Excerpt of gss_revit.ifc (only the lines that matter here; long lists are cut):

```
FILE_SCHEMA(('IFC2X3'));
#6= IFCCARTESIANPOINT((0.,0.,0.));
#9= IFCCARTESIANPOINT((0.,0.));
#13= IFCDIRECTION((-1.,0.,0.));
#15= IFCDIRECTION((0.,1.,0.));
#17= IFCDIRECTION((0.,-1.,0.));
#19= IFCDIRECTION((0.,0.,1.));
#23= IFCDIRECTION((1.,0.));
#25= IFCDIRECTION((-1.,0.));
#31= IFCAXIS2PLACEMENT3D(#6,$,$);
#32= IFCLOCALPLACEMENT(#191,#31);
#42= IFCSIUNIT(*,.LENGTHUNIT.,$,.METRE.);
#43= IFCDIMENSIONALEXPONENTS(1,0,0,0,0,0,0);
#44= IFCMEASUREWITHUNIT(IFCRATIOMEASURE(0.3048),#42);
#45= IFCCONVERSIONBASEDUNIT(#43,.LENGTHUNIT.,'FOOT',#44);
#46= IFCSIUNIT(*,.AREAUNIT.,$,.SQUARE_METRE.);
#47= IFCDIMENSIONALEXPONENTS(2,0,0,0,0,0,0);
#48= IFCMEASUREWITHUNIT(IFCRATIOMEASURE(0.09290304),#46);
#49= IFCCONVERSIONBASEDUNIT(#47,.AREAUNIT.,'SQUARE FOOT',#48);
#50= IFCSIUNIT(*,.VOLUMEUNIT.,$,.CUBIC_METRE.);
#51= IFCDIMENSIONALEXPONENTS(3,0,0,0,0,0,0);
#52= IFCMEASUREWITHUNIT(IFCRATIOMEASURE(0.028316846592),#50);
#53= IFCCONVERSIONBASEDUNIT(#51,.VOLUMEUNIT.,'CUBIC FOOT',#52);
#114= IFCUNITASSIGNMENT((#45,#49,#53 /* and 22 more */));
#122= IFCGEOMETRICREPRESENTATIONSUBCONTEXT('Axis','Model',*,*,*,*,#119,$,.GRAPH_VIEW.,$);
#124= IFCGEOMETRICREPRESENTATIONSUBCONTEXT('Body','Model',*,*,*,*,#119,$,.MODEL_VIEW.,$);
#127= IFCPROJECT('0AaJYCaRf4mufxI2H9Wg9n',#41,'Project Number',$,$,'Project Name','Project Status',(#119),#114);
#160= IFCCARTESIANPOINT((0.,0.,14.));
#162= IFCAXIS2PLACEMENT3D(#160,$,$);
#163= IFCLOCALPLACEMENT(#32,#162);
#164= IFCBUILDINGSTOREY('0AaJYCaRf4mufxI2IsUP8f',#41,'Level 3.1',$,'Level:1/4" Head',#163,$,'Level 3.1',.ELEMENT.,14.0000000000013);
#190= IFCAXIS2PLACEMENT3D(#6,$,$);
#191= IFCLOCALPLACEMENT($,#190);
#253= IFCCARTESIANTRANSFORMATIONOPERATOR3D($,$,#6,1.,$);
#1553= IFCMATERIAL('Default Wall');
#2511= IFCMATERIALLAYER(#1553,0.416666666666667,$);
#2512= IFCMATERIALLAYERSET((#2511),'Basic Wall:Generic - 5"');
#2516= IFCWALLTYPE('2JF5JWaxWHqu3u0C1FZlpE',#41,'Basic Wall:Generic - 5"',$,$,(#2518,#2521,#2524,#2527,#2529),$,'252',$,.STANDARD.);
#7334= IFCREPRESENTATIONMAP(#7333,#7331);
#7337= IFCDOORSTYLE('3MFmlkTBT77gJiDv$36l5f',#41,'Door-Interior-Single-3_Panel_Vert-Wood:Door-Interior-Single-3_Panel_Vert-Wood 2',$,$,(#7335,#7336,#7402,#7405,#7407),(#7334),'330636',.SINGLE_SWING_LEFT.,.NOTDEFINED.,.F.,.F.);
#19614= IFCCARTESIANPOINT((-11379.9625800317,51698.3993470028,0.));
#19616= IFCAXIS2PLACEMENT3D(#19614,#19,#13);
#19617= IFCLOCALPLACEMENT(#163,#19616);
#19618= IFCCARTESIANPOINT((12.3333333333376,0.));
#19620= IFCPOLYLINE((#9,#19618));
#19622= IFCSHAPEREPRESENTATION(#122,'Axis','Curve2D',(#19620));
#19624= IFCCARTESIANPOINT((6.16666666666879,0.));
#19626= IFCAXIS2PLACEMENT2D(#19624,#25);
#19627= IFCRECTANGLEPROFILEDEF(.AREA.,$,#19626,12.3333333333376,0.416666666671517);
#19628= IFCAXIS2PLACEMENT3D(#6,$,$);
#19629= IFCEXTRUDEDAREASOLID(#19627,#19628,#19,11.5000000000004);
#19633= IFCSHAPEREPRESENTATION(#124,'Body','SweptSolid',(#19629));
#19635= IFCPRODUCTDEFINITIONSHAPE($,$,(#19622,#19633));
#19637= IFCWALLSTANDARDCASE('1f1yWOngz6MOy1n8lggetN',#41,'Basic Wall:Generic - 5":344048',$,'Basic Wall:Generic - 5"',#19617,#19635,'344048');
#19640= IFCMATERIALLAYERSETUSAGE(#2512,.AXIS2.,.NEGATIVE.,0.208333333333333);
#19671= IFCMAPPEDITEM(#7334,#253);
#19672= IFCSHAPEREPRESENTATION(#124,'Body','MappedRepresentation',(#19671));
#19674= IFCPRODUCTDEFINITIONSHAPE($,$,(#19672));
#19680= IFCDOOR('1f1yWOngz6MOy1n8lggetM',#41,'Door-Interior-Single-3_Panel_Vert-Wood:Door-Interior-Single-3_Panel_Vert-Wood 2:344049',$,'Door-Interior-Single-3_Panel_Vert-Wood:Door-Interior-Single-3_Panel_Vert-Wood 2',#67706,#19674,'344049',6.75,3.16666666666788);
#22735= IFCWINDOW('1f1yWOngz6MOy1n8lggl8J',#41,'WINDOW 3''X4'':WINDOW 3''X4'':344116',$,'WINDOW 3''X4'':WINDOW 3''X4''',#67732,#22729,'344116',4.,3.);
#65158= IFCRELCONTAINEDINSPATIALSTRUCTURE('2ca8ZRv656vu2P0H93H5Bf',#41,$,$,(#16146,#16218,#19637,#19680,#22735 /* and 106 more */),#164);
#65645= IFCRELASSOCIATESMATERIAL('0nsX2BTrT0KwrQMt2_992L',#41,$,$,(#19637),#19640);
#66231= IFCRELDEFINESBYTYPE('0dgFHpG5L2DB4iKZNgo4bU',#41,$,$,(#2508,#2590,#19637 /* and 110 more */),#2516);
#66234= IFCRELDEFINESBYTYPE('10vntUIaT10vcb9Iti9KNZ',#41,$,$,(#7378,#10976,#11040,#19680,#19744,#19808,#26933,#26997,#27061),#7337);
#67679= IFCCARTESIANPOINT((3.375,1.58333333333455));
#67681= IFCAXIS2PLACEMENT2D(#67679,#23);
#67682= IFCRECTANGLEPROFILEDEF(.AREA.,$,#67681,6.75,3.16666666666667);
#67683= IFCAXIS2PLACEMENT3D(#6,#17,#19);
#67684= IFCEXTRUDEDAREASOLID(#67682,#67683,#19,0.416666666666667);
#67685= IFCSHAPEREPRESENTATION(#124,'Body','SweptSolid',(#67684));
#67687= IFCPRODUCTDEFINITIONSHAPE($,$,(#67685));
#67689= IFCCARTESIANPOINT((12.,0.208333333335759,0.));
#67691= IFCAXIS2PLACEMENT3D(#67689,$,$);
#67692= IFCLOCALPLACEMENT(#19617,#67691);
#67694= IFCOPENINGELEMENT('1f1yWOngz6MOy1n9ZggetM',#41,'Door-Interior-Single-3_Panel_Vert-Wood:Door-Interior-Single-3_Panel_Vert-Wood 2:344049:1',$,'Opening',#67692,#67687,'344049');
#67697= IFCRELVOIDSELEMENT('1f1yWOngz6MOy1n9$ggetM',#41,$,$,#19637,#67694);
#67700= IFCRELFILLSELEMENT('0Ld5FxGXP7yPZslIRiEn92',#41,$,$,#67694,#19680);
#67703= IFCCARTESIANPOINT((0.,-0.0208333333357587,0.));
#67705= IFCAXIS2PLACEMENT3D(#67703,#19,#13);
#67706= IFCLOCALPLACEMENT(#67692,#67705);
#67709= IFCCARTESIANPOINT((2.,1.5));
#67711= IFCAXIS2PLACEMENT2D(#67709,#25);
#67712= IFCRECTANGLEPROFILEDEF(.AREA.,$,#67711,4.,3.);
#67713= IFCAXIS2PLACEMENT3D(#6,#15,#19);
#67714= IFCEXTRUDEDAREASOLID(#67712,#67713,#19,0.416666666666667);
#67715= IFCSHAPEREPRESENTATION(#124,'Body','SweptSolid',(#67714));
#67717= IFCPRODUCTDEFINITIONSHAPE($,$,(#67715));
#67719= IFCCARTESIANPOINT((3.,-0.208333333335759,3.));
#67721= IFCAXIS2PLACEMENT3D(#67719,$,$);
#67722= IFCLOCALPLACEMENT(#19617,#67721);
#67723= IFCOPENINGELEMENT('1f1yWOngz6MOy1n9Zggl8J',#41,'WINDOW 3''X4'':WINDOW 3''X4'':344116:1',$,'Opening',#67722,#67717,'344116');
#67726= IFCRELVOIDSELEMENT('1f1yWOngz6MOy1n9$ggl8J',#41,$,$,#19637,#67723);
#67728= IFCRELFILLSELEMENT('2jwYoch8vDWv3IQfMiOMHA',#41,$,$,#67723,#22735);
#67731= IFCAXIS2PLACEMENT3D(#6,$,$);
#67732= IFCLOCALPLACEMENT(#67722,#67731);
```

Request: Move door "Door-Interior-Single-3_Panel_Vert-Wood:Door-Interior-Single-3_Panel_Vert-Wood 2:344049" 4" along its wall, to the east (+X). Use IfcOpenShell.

```python
import ifcopenshell
import ifcopenshell.api.geometry
import ifcopenshell.util.placement
import ifcopenshell.util.unit

model = ifcopenshell.open("gss_revit.ifc")
unit_scale = ifcopenshell.util.unit.calculate_unit_scale(model)

door = model.by_guid("1f1yWOngz6MOy1n8lggetM")
opening = door.FillsVoids[0].RelatingOpeningElement
wall = opening.VoidsElements[0].RelatingBuildingElement

wall_matrix = ifcopenshell.util.placement.get_local_placement(wall.ObjectPlacement)
shift = wall_matrix[:3, 0] * -4 * 0.0254 / unit_scale
before = ifcopenshell.util.placement.get_local_placement(door.ObjectPlacement)[:3, 3].copy()

# The door is placed relative to its opening, so it follows when the opening moves.
matrix = ifcopenshell.util.placement.get_local_placement(opening.ObjectPlacement)
matrix[:3, 3] += shift
ifcopenshell.api.geometry.edit_object_placement(
    model, product=opening, matrix=matrix, is_si=False, should_transform_children=True
)

after = ifcopenshell.util.placement.get_local_placement(door.ObjectPlacement)[:3, 3]
print("door moved by", (after - before).round(3) + 0.0)

model.write("gss_revit_rev.ifc")
```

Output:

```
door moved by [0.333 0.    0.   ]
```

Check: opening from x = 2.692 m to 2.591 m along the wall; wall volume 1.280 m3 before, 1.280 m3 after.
